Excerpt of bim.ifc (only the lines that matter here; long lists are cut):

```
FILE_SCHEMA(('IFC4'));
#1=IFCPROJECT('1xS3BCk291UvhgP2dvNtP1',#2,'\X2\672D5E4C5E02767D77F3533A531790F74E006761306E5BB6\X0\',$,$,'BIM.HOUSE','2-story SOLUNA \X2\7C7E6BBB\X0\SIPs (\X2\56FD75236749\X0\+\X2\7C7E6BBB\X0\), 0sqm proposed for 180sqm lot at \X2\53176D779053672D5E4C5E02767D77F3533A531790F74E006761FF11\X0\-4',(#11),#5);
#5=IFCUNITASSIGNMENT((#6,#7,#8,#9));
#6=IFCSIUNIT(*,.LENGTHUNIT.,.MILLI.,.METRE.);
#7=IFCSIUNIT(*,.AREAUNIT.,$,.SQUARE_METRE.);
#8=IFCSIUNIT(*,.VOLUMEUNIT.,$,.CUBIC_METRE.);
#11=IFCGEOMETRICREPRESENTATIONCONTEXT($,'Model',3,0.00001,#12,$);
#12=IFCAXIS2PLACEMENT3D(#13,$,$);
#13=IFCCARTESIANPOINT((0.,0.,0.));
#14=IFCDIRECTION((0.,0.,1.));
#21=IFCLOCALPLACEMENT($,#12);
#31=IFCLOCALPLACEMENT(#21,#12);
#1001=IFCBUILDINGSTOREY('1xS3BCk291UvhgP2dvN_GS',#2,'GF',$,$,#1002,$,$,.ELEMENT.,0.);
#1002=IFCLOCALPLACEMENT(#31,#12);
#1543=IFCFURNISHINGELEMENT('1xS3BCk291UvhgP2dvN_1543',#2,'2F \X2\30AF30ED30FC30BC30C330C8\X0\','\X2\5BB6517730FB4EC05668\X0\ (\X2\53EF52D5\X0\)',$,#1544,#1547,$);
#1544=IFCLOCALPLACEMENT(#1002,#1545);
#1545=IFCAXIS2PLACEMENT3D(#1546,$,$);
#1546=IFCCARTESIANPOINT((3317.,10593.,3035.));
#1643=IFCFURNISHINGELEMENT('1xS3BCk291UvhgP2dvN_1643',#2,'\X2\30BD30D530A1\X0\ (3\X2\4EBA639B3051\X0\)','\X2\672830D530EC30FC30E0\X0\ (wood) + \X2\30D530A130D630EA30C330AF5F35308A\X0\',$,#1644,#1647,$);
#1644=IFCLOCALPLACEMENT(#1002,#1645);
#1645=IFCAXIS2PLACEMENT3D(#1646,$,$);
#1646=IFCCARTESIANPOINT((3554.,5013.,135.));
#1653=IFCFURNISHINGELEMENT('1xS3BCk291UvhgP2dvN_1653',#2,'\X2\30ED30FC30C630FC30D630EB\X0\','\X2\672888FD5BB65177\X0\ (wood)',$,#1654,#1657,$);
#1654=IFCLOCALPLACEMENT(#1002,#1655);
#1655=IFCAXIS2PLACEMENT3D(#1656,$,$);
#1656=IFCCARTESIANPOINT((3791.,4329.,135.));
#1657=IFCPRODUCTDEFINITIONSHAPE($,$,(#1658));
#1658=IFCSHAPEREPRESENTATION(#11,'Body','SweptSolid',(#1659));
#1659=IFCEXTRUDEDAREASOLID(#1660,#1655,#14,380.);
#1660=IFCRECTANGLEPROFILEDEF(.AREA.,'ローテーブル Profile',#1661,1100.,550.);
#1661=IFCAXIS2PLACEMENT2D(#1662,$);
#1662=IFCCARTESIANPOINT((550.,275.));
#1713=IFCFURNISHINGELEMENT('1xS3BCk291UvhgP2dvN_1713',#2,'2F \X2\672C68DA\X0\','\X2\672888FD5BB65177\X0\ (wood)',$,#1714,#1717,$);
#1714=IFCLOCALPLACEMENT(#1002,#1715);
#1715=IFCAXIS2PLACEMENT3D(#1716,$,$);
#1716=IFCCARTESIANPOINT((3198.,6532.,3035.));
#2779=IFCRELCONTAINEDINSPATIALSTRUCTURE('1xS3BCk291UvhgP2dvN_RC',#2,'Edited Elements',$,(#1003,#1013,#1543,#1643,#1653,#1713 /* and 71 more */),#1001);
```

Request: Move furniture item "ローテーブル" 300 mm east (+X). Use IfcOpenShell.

```python
import ifcopenshell
import ifcopenshell.api.geometry
import ifcopenshell.util.placement
import ifcopenshell.util.unit

model = ifcopenshell.open("bim.ifc")
unit_scale = ifcopenshell.util.unit.calculate_unit_scale(model)

item = model.by_guid("1xS3BCk291UvhgP2dvN_1653")
matrix = ifcopenshell.util.placement.get_local_placement(item.ObjectPlacement)
matrix[0, 3] += 0.3 / unit_scale
ifcopenshell.api.geometry.edit_object_placement(model, product=item, matrix=matrix, is_si=False)

print(ifcopenshell.util.placement.get_local_placement(item.ObjectPlacement).round(3) + 0.0)

model.write("bim-out.ifc")
```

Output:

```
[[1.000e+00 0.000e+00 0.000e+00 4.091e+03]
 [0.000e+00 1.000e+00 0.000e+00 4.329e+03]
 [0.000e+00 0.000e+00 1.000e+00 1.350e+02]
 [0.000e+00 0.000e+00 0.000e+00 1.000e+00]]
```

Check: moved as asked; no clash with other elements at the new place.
